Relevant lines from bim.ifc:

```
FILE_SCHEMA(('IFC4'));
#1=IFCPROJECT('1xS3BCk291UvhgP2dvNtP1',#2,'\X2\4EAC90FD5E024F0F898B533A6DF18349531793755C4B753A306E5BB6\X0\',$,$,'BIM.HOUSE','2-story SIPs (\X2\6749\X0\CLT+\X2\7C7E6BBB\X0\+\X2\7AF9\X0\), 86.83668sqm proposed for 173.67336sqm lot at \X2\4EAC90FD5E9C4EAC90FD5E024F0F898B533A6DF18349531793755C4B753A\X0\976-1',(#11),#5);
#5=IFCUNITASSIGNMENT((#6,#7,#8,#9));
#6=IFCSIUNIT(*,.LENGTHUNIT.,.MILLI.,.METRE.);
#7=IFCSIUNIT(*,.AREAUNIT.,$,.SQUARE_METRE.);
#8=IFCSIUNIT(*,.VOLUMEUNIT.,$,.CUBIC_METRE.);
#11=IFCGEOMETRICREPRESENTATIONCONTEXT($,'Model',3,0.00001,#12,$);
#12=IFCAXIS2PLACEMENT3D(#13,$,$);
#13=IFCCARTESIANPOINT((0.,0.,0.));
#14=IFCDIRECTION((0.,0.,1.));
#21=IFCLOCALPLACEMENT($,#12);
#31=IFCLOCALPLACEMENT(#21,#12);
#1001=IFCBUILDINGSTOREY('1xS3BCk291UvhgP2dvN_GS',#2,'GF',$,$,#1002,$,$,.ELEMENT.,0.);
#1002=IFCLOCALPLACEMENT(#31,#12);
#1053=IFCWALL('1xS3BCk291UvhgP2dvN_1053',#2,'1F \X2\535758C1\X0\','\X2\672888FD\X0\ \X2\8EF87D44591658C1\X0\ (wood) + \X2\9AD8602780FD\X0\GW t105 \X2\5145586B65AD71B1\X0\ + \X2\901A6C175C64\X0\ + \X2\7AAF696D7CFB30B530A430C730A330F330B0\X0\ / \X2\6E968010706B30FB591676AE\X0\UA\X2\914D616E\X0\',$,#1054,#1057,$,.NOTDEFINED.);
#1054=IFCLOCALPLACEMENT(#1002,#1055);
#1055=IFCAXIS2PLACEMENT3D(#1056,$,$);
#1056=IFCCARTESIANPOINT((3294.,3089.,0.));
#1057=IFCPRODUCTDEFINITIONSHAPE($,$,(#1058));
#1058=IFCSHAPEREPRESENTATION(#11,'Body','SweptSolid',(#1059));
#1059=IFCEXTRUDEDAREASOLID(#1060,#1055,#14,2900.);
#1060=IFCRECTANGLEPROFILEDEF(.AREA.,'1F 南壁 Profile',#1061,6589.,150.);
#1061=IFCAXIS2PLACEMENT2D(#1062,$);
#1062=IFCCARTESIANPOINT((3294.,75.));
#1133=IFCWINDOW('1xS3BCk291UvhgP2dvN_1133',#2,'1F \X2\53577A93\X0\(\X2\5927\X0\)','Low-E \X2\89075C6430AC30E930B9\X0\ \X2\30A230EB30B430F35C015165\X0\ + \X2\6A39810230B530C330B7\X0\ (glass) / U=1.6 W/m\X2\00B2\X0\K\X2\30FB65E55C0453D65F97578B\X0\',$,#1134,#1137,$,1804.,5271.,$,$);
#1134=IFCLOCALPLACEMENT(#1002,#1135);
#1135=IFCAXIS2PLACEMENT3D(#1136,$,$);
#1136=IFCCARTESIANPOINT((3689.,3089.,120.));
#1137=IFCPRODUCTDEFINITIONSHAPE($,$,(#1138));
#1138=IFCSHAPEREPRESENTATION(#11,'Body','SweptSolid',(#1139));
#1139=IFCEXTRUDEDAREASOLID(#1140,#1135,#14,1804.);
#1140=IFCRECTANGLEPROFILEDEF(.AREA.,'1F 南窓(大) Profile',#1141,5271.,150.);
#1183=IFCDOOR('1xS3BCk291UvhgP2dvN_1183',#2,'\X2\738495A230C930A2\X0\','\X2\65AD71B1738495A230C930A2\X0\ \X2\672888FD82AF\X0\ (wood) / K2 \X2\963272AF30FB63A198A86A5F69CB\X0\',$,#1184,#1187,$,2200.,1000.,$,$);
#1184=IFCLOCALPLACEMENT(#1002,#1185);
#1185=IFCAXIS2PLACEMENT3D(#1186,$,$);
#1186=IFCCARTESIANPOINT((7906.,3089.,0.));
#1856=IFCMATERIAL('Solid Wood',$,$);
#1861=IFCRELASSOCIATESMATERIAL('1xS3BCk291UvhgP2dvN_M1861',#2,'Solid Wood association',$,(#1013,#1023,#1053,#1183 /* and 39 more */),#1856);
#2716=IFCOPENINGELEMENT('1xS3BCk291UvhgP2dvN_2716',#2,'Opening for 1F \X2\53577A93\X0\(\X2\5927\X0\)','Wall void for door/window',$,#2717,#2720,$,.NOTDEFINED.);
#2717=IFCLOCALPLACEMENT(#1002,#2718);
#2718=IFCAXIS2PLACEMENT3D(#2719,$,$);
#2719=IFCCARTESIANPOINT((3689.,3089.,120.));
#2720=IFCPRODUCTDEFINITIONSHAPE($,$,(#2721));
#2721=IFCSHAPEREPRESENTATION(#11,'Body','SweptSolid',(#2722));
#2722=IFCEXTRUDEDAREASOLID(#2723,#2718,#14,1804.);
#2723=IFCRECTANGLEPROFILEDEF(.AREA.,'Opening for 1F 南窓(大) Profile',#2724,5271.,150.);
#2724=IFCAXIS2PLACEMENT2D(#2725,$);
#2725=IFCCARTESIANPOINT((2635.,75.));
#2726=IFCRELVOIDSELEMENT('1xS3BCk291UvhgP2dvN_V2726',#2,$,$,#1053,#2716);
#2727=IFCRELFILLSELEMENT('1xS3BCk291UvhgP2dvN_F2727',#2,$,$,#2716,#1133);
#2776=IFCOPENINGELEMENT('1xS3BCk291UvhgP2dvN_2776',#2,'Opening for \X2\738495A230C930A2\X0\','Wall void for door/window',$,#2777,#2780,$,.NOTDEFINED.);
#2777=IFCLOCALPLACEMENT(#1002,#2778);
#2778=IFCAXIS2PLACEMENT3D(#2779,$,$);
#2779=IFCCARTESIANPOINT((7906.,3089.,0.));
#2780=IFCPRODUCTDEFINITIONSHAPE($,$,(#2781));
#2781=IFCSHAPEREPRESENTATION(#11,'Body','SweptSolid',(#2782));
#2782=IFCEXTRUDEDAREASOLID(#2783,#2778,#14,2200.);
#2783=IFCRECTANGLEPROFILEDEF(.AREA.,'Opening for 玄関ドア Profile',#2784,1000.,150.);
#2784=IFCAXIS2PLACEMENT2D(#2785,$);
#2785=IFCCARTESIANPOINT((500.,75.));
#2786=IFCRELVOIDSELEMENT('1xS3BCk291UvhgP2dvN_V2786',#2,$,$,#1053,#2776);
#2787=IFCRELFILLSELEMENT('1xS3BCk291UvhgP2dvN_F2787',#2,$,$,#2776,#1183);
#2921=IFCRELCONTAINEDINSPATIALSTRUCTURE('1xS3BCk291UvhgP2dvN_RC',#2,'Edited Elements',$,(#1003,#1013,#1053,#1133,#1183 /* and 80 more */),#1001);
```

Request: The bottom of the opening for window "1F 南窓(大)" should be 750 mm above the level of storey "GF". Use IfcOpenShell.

```python
import numpy as np
import ifcopenshell
import ifcopenshell.api.geometry
import ifcopenshell.geom
import ifcopenshell.util.element
import ifcopenshell.util.placement
import ifcopenshell.util.shape
import ifcopenshell.util.unit

model = ifcopenshell.open("bim.ifc")
unit_scale = ifcopenshell.util.unit.calculate_unit_scale(model)

window = model.by_guid("1xS3BCk291UvhgP2dvN_1133")
opening = window.FillsVoids[0].RelatingOpeningElement
storey = ifcopenshell.util.element.get_container(window, ifc_class="IfcBuildingStorey")
level = ifcopenshell.util.placement.get_local_placement(storey.ObjectPlacement)[2, 3]

# The opening's origin need not be at the sill, so measure its lowest point.
shape = ifcopenshell.geom.create_shape(ifcopenshell.geom.settings(), opening)
bottom = ifcopenshell.util.shape.get_shape_bottom_elevation(shape, shape.geometry) / unit_scale
dz = level + 750.0 - bottom

shift = np.array([0.0, 0.0, dz])
# The window is not placed relative to its opening, so move both.
for product in (opening, window):
    matrix = ifcopenshell.util.placement.get_local_placement(product.ObjectPlacement)
    matrix[:3, 3] += shift
    ifcopenshell.api.geometry.edit_object_placement(model, product=product, matrix=matrix, is_si=False)

print(f"moved by {dz * unit_scale:+.3f} m")

model.write("bim_v2.ifc")
```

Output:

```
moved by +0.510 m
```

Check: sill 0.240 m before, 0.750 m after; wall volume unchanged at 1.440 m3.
